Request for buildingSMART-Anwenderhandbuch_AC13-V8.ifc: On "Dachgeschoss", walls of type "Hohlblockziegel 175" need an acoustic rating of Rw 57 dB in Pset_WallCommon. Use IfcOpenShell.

First a look at what the model holds.

```python
import ifcopenshell
import ifcopenshell.util.element

model = ifcopenshell.open("buildingSMART-Anwenderhandbuch_AC13-V8.ifc")
print(model.schema)
storey = next(s for s in model.by_type("IfcBuildingStorey") if s.Name == "Dachgeschoss")
walls = [e for e in ifcopenshell.util.element.get_decomposition(storey) if e.is_a("IfcWall")]
seen = {}
for e in walls:
    element_type = ifcopenshell.util.element.get_type(e)
    key = (element_type.Name if element_type != e and element_type else None, ifcopenshell.util.element.get_pset(e, "Pset_WallCommon", "AcousticRating"))
    seen[key] = seen.get(key, 0) + 1
for (name, value), count in sorted(seen.items(), key=str):
    print(count, "x", name, "|", value)
```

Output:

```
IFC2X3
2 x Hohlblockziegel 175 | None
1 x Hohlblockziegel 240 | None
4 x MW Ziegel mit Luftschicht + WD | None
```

```python
import ifcopenshell
import ifcopenshell.api.pset
import ifcopenshell.util.element

model = ifcopenshell.open("buildingSMART-Anwenderhandbuch_AC13-V8.ifc")

storey = next(s for s in model.by_type("IfcBuildingStorey") if s.Name == "Dachgeschoss")
walls = [e for e in ifcopenshell.util.element.get_decomposition(storey) if e.is_a("IfcWall")]

count = 0
for e in walls:
    element_type = ifcopenshell.util.element.get_type(e)
    if element_type in (None, e) or element_type.Name != "Hohlblockziegel 175":
        continue
    # add_pset returns the element's existing set when there is one.
    pset = ifcopenshell.api.pset.add_pset(model, product=e, name="Pset_WallCommon")
    ifcopenshell.api.pset.edit_pset(model, pset=pset, properties={"AcousticRating": "Rw 57 dB"})
    count += 1

print(count, "walls updated")

model.write("buildingSMART-Anwenderhandbuch_AC13-V8_rev.ifc")
```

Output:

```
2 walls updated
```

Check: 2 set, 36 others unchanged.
